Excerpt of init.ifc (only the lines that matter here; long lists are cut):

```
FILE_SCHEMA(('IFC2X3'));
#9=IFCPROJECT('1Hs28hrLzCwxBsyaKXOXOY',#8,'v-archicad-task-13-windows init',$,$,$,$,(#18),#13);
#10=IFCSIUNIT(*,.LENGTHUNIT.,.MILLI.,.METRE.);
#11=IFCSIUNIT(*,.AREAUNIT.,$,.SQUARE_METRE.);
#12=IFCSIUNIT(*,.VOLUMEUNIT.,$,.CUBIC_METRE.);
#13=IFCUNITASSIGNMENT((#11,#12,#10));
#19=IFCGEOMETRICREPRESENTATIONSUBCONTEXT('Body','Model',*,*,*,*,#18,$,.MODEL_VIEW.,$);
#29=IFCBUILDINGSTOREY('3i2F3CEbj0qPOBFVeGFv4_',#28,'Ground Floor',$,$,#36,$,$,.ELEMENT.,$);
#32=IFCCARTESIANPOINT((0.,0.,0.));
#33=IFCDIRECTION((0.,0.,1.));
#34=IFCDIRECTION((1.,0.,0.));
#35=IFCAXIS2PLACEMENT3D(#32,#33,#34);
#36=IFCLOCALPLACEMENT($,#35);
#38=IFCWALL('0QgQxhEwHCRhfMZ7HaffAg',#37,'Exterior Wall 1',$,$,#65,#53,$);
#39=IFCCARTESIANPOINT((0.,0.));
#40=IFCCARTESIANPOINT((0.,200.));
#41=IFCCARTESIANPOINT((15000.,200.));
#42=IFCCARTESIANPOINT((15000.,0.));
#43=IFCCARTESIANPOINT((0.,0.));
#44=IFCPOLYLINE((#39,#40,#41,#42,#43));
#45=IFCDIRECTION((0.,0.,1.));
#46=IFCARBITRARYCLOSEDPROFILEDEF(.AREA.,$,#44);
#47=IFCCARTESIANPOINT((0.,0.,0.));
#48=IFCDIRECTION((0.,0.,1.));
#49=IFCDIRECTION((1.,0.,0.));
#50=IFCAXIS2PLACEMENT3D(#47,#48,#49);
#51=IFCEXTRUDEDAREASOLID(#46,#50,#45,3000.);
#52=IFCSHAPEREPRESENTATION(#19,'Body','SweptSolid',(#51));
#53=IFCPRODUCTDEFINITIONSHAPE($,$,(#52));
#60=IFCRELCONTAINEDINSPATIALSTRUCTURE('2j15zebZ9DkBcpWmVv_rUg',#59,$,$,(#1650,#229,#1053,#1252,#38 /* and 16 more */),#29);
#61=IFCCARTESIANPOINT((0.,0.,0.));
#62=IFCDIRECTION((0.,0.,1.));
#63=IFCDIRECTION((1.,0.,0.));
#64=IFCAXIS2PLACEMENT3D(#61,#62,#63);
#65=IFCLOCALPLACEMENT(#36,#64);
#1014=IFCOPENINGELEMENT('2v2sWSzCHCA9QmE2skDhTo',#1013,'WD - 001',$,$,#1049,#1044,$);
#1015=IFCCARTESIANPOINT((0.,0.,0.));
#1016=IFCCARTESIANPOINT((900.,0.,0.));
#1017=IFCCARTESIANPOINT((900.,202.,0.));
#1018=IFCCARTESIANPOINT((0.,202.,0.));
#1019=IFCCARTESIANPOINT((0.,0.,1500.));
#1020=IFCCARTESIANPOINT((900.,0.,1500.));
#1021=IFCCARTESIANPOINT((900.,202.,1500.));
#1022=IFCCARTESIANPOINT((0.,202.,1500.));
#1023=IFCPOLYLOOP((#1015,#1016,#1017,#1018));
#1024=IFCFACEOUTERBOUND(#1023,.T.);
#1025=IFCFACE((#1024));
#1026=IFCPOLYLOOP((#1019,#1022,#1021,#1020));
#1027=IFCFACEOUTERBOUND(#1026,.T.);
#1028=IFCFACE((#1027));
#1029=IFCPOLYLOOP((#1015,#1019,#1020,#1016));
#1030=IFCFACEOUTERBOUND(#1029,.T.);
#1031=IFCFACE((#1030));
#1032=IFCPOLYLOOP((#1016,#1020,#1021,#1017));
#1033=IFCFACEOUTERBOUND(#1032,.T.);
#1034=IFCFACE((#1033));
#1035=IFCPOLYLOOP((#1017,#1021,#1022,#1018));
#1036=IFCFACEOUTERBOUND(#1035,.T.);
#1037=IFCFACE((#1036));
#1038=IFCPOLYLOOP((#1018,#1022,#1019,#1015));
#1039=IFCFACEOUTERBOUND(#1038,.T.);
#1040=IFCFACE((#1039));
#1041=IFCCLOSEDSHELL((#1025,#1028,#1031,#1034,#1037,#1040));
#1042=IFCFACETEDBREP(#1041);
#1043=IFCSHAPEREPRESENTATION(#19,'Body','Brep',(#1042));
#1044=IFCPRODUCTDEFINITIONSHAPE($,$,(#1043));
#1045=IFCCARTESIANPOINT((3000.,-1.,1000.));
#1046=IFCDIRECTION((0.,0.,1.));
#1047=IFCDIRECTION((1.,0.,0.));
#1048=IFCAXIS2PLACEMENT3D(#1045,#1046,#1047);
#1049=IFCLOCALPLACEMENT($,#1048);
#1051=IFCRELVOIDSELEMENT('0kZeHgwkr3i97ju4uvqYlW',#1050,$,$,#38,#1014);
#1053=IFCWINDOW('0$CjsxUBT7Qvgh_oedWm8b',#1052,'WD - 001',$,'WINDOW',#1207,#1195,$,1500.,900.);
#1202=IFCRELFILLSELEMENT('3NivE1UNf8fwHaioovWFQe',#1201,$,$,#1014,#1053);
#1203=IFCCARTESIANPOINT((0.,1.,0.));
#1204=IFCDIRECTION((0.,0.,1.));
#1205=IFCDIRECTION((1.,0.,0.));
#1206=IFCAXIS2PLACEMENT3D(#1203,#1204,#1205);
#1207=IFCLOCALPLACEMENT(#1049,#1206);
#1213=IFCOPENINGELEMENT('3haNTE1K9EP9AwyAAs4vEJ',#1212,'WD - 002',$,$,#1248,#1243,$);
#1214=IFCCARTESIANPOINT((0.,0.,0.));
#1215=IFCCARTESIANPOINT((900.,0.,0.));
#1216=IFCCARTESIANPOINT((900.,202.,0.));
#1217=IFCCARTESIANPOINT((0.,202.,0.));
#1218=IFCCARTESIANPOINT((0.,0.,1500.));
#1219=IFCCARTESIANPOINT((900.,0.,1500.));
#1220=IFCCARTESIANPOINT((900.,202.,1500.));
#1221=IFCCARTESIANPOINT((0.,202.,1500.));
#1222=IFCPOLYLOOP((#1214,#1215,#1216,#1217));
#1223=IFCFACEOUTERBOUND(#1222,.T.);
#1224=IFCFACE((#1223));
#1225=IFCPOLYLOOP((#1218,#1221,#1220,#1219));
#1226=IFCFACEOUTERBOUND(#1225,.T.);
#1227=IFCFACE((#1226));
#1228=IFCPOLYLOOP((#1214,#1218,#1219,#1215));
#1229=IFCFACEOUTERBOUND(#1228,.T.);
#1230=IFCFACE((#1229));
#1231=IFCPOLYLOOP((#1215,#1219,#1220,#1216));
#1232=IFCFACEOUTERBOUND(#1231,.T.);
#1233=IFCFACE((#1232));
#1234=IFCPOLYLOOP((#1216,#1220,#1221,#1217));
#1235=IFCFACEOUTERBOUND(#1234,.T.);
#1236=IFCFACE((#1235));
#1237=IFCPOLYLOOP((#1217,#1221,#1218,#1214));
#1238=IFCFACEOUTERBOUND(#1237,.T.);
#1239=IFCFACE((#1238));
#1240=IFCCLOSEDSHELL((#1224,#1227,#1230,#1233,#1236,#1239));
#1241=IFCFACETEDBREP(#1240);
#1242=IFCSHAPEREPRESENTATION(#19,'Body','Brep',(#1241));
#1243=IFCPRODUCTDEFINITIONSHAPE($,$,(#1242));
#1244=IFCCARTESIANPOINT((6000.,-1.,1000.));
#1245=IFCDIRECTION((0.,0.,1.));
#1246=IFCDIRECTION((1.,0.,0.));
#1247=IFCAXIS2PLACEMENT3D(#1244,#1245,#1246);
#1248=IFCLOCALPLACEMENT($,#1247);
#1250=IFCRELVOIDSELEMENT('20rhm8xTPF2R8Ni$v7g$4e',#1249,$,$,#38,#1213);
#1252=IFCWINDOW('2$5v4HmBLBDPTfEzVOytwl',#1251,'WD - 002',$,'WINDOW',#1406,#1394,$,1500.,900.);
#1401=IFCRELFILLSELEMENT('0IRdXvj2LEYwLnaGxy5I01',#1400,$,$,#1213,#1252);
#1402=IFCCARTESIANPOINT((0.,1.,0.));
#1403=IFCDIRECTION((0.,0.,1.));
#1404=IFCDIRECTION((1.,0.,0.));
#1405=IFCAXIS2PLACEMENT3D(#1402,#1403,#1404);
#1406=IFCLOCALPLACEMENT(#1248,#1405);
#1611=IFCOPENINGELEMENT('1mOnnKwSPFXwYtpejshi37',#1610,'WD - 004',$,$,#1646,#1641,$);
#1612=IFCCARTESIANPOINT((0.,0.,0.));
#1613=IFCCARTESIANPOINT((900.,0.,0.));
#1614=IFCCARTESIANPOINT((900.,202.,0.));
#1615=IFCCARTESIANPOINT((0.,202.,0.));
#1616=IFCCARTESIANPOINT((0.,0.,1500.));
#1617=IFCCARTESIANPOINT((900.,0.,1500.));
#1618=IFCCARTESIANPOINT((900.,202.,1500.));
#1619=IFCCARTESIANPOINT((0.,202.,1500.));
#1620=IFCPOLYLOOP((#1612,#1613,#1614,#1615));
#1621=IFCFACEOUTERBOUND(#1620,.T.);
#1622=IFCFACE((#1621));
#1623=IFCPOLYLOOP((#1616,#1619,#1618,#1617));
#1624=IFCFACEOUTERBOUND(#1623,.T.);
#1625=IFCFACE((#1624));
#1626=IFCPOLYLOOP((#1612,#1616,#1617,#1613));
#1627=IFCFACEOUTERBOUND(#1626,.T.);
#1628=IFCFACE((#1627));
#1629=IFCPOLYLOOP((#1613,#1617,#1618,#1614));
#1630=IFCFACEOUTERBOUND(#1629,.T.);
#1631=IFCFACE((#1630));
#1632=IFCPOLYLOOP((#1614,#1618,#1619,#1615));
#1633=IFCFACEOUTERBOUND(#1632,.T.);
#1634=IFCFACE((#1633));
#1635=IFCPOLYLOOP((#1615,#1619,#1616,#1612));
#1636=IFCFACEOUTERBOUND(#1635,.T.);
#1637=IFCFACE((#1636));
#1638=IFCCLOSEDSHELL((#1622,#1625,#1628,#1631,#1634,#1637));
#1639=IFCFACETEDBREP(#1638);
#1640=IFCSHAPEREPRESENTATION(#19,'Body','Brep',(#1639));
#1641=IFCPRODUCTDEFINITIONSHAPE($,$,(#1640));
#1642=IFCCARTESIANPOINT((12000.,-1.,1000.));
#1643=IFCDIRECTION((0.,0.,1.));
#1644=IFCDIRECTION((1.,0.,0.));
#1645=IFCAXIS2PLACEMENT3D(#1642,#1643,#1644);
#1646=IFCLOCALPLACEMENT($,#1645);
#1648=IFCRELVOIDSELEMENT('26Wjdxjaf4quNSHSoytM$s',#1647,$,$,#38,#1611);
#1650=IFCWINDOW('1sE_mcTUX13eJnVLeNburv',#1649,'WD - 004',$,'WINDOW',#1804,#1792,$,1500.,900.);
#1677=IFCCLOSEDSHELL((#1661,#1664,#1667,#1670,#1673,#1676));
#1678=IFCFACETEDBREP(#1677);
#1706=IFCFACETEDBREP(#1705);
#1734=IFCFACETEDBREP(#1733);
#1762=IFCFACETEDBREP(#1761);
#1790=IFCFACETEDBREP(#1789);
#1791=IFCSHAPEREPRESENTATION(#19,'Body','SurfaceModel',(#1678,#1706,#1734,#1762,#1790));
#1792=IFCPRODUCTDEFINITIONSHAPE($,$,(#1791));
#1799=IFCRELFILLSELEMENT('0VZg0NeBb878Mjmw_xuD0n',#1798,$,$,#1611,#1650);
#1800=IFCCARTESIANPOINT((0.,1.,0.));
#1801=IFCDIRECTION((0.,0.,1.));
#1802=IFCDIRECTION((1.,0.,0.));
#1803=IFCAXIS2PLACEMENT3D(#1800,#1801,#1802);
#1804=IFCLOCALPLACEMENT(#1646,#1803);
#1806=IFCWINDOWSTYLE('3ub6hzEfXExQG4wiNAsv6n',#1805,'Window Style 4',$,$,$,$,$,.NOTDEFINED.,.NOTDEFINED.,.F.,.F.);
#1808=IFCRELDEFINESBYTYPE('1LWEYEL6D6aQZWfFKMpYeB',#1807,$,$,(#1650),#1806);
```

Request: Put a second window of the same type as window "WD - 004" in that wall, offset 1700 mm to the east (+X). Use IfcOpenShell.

```python
import ifcopenshell
import ifcopenshell.api.feature
import ifcopenshell.api.geometry
import ifcopenshell.api.root
import ifcopenshell.geom
import ifcopenshell.util.element
import ifcopenshell.util.placement
import ifcopenshell.util.shape
import ifcopenshell.util.unit

model = ifcopenshell.open("init.ifc")
unit_scale = ifcopenshell.util.unit.calculate_unit_scale(model)
settings = ifcopenshell.geom.settings()


def volume(element):
    """Net volume in cubic metres, openings subtracted."""
    shape = ifcopenshell.geom.create_shape(settings, element)
    return ifcopenshell.util.shape.get_volume(shape.geometry)


window = model.by_guid("1sE_mcTUX13eJnVLeNburv")
opening = window.FillsVoids[0].RelatingOpeningElement
wall = opening.VoidsElements[0].RelatingBuildingElement
before = volume(wall)
shift = ifcopenshell.util.placement.get_local_placement(wall.ObjectPlacement)[:3, 0] * 1.7 / unit_scale

# copy_class copies the void relationship, type, container and properties, but no geometry.
new_opening = ifcopenshell.api.root.copy_class(model, product=opening)
new_opening.Representation = ifcopenshell.util.element.copy_deep(
    model, opening.Representation, exclude=["IfcGeometricRepresentationContext", "IfcRepresentationMap"]
)
new_window = ifcopenshell.api.root.copy_class(model, product=window)
new_window.Representation = ifcopenshell.util.element.copy_deep(
    model, window.Representation, exclude=["IfcGeometricRepresentationContext", "IfcRepresentationMap"]
)
fills = ifcopenshell.api.feature.add_filling(model, opening=new_opening, element=new_window)
fills.OwnerHistory = new_window.OwnerHistory  # required in IFC2X3

for old, new in ((opening, new_opening), (window, new_window)):
    matrix = ifcopenshell.util.placement.get_local_placement(old.ObjectPlacement)
    matrix[:3, 3] += shift
    ifcopenshell.api.geometry.edit_object_placement(model, product=new, matrix=matrix, is_si=False)

after = volume(wall)

print(f"wall volume {before:.3f} -> {after:.3f} m3")

model.write("init_updated.ifc")
```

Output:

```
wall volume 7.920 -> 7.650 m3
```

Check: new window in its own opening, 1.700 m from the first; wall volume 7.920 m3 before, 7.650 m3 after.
